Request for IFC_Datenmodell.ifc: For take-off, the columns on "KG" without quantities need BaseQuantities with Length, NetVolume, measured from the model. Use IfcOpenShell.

First a look at what the model holds.

```python
import ifcopenshell
import ifcopenshell.util.element
import ifcopenshell.util.unit

model = ifcopenshell.open("IFC_Datenmodell.ifc")
print(model.schema)
for unit_type in ("LENGTHUNIT", "AREAUNIT", "VOLUMEUNIT"):
    print(unit_type, ifcopenshell.util.unit.calculate_unit_scale(model, unit_type))
storey = next(s for s in model.by_type("IfcBuildingStorey") if s.Name == "KG")
columns = [e for e in ifcopenshell.util.element.get_decomposition(storey) if e.is_a("IfcColumn")]
for e in sorted(columns, key=lambda e: e.id()):
    print(e.id(), e.is_a(), e.Name, list(ifcopenshell.util.element.get_psets(e, qtos_only=True)), sep=" | ")
```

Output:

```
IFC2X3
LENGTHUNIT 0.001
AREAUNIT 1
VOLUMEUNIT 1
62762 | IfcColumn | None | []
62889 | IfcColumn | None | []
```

```python
import ifcopenshell
import ifcopenshell.api.pset
import ifcopenshell.geom
import ifcopenshell.util.element
import ifcopenshell.util.shape
import ifcopenshell.util.unit

model = ifcopenshell.open("IFC_Datenmodell.ifc")
unit_scale = ifcopenshell.util.unit.calculate_unit_scale(model)
volume_scale = ifcopenshell.util.unit.calculate_unit_scale(model, "VOLUMEUNIT")
settings = ifcopenshell.geom.settings()

storey = next(s for s in model.by_type("IfcBuildingStorey") if s.Name == "KG")
columns = [e for e in ifcopenshell.util.element.get_decomposition(storey) if e.is_a("IfcColumn")]

for e in sorted(columns, key=lambda e: e.id()):
    if ifcopenshell.util.element.get_psets(e, qtos_only=True, should_inherit=False):
        continue
    # Geometry comes back in metres, in the element's own axes.
    shape = ifcopenshell.geom.create_shape(settings, e)
    values = {
        "Length": ifcopenshell.util.shape.get_z(shape.geometry) / unit_scale,
        "NetVolume": ifcopenshell.util.shape.get_volume(shape.geometry) / volume_scale,
    }
    qto = ifcopenshell.api.pset.add_qto(model, product=e, name="BaseQuantities")
    ifcopenshell.api.pset.edit_qto(model, qto=qto, properties=values)
    print(e.id(), {k: round(v, 3) for k, v in values.items()})

model.write("IFC_Datenmodell-out.ifc")
```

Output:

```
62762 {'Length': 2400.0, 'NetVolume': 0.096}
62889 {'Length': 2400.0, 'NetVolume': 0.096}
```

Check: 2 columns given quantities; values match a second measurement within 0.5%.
